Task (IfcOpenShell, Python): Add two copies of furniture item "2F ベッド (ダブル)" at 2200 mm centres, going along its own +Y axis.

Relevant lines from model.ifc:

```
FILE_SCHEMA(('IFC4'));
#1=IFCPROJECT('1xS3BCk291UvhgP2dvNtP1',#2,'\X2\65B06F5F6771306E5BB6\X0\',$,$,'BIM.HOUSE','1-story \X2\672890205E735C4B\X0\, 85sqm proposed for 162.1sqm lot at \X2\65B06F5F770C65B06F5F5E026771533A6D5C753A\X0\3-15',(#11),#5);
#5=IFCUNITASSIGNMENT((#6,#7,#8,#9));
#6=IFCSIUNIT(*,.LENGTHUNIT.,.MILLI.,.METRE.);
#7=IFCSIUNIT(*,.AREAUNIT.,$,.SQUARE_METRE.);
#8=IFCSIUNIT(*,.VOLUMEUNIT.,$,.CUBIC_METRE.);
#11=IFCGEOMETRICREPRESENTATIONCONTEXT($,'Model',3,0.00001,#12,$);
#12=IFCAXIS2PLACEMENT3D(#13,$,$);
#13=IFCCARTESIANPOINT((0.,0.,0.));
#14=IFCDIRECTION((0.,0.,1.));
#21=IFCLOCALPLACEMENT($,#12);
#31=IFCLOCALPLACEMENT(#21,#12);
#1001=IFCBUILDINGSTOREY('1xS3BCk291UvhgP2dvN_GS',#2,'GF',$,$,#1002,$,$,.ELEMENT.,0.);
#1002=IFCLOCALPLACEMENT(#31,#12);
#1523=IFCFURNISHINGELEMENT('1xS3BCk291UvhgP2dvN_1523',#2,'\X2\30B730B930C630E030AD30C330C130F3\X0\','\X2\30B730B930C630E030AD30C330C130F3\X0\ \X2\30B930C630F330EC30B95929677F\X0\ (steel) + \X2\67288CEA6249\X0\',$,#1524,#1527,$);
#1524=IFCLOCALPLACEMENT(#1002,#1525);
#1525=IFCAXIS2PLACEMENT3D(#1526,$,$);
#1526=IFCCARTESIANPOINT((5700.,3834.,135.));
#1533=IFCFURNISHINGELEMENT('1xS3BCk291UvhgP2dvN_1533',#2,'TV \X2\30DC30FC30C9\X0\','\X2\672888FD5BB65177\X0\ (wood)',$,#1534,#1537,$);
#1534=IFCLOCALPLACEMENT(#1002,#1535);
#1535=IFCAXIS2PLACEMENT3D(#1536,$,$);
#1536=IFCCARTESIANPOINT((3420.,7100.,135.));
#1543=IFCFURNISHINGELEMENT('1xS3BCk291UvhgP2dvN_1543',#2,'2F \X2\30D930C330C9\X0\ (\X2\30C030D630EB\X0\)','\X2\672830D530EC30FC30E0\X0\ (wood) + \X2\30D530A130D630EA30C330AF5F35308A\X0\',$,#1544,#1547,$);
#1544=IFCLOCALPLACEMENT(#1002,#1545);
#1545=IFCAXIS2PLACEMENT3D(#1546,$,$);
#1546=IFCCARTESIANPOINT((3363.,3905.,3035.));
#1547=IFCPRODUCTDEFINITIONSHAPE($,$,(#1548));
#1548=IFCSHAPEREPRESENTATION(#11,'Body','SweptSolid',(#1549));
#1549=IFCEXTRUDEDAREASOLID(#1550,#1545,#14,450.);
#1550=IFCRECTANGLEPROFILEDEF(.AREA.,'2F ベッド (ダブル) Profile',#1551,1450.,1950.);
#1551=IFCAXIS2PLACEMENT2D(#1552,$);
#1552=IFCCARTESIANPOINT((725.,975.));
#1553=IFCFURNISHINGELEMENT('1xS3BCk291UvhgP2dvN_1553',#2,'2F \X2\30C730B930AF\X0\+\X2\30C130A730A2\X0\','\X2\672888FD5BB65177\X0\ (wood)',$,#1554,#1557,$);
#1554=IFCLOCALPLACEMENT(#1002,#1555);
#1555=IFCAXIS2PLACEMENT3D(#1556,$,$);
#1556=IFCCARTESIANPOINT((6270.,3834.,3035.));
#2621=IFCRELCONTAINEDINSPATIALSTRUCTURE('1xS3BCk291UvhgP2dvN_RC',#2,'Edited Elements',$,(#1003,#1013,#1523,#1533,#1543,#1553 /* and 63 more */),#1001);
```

```python
import ifcopenshell
import ifcopenshell.api.geometry
import ifcopenshell.api.root
import ifcopenshell.util.element
import ifcopenshell.util.placement

model = ifcopenshell.open("model.ifc")


def reuse_history(source, copy):
    """copy_class also copies each property set's owner history, people and application; keep the originals."""
    for rel in copy.IsDefinedBy:
        if rel.is_a("IfcRelDefinesByProperties") and (history := rel.RelatingPropertyDefinition.OwnerHistory):
            rel.RelatingPropertyDefinition.OwnerHistory = source.OwnerHistory
            ifcopenshell.util.element.remove_deep2(model, history)


source = model.by_guid("1xS3BCk291UvhgP2dvN_1543")
base = ifcopenshell.util.placement.get_local_placement(source.ObjectPlacement)
step = base[:3, 1] * 2200.0

for i in range(1, 3):
    copy = ifcopenshell.api.root.copy_class(model, product=source)
    copy.Representation = ifcopenshell.util.element.copy_deep(
        model, source.Representation, exclude=["IfcGeometricRepresentationContext", "IfcRepresentationMap"]
    )
    reuse_history(source, copy)
    matrix = base.copy()
    matrix[:3, 3] += i * step
    print("added at", matrix[:3, 3].round(3) + 0.0)
    ifcopenshell.api.geometry.edit_object_placement(model, product=copy, matrix=matrix, is_si=False)

model.write("model_v2.ifc")
```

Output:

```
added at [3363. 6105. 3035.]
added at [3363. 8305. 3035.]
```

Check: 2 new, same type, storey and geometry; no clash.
